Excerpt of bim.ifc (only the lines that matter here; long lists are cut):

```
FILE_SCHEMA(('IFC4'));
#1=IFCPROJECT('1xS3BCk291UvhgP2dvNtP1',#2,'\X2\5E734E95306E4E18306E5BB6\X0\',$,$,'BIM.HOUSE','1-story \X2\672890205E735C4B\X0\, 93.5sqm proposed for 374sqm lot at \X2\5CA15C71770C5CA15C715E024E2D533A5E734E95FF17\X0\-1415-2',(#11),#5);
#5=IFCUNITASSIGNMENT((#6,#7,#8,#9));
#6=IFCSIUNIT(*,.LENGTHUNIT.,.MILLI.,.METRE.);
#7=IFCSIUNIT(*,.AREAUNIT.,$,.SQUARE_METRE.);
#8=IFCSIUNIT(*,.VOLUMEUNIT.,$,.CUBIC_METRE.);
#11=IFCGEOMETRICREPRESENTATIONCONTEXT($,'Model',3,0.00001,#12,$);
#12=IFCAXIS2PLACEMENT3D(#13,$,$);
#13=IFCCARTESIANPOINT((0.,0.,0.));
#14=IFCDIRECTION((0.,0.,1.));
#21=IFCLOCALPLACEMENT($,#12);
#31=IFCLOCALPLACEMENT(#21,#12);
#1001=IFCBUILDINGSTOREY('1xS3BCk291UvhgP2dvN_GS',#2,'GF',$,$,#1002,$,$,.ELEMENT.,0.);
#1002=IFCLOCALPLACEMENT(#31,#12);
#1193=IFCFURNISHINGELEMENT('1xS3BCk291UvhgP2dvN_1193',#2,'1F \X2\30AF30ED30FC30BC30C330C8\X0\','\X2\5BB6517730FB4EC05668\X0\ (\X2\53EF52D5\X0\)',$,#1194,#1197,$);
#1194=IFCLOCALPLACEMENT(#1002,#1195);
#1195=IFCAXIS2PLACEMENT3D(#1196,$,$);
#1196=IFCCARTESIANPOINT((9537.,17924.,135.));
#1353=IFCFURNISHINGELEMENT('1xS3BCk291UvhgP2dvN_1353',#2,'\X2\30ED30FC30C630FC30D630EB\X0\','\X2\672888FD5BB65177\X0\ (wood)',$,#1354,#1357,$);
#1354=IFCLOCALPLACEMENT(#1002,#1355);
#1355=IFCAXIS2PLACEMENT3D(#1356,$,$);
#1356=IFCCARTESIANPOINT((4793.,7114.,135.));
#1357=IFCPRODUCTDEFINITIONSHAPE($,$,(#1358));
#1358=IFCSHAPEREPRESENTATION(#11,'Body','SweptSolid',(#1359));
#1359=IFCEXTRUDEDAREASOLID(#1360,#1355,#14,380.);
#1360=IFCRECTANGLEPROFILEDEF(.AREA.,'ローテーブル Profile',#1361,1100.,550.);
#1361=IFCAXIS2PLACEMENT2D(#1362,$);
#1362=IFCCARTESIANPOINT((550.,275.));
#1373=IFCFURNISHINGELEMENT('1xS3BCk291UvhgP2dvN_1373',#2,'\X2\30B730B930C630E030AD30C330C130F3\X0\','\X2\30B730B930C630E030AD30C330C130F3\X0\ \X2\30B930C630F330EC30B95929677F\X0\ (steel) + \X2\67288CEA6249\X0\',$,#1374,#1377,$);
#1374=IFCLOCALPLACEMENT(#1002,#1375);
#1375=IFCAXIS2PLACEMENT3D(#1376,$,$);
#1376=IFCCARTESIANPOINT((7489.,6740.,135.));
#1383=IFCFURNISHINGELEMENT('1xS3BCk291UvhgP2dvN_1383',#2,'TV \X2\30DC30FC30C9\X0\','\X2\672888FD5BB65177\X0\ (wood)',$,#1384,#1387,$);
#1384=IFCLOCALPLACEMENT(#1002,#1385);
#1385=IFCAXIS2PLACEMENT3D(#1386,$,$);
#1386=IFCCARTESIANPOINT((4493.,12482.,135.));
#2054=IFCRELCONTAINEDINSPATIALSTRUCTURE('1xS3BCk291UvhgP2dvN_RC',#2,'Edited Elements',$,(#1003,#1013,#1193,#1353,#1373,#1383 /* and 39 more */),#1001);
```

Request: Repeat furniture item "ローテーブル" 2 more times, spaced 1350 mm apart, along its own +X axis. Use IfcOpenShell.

```python
import ifcopenshell
import ifcopenshell.api.geometry
import ifcopenshell.api.root
import ifcopenshell.util.element
import ifcopenshell.util.placement

model = ifcopenshell.open("bim.ifc")


def reuse_history(source, copy):
    """copy_class also copies each property set's owner history, people and application; keep the originals."""
    for rel in copy.IsDefinedBy:
        if rel.is_a("IfcRelDefinesByProperties") and (history := rel.RelatingPropertyDefinition.OwnerHistory):
            rel.RelatingPropertyDefinition.OwnerHistory = source.OwnerHistory
            ifcopenshell.util.element.remove_deep2(model, history)


source = model.by_guid("1xS3BCk291UvhgP2dvN_1353")
base = ifcopenshell.util.placement.get_local_placement(source.ObjectPlacement)
step = base[:3, 0] * 1350.0

for i in range(1, 3):
    copy = ifcopenshell.api.root.copy_class(model, product=source)
    copy.Representation = ifcopenshell.util.element.copy_deep(
        model, source.Representation, exclude=["IfcGeometricRepresentationContext", "IfcRepresentationMap"]
    )
    reuse_history(source, copy)
    matrix = base.copy()
    matrix[:3, 3] += i * step
    print("added at", matrix[:3, 3].round(3) + 0.0)
    ifcopenshell.api.geometry.edit_object_placement(model, product=copy, matrix=matrix, is_si=False)

model.write("bim_v2.ifc")
```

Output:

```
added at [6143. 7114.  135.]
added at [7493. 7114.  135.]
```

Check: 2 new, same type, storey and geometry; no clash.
